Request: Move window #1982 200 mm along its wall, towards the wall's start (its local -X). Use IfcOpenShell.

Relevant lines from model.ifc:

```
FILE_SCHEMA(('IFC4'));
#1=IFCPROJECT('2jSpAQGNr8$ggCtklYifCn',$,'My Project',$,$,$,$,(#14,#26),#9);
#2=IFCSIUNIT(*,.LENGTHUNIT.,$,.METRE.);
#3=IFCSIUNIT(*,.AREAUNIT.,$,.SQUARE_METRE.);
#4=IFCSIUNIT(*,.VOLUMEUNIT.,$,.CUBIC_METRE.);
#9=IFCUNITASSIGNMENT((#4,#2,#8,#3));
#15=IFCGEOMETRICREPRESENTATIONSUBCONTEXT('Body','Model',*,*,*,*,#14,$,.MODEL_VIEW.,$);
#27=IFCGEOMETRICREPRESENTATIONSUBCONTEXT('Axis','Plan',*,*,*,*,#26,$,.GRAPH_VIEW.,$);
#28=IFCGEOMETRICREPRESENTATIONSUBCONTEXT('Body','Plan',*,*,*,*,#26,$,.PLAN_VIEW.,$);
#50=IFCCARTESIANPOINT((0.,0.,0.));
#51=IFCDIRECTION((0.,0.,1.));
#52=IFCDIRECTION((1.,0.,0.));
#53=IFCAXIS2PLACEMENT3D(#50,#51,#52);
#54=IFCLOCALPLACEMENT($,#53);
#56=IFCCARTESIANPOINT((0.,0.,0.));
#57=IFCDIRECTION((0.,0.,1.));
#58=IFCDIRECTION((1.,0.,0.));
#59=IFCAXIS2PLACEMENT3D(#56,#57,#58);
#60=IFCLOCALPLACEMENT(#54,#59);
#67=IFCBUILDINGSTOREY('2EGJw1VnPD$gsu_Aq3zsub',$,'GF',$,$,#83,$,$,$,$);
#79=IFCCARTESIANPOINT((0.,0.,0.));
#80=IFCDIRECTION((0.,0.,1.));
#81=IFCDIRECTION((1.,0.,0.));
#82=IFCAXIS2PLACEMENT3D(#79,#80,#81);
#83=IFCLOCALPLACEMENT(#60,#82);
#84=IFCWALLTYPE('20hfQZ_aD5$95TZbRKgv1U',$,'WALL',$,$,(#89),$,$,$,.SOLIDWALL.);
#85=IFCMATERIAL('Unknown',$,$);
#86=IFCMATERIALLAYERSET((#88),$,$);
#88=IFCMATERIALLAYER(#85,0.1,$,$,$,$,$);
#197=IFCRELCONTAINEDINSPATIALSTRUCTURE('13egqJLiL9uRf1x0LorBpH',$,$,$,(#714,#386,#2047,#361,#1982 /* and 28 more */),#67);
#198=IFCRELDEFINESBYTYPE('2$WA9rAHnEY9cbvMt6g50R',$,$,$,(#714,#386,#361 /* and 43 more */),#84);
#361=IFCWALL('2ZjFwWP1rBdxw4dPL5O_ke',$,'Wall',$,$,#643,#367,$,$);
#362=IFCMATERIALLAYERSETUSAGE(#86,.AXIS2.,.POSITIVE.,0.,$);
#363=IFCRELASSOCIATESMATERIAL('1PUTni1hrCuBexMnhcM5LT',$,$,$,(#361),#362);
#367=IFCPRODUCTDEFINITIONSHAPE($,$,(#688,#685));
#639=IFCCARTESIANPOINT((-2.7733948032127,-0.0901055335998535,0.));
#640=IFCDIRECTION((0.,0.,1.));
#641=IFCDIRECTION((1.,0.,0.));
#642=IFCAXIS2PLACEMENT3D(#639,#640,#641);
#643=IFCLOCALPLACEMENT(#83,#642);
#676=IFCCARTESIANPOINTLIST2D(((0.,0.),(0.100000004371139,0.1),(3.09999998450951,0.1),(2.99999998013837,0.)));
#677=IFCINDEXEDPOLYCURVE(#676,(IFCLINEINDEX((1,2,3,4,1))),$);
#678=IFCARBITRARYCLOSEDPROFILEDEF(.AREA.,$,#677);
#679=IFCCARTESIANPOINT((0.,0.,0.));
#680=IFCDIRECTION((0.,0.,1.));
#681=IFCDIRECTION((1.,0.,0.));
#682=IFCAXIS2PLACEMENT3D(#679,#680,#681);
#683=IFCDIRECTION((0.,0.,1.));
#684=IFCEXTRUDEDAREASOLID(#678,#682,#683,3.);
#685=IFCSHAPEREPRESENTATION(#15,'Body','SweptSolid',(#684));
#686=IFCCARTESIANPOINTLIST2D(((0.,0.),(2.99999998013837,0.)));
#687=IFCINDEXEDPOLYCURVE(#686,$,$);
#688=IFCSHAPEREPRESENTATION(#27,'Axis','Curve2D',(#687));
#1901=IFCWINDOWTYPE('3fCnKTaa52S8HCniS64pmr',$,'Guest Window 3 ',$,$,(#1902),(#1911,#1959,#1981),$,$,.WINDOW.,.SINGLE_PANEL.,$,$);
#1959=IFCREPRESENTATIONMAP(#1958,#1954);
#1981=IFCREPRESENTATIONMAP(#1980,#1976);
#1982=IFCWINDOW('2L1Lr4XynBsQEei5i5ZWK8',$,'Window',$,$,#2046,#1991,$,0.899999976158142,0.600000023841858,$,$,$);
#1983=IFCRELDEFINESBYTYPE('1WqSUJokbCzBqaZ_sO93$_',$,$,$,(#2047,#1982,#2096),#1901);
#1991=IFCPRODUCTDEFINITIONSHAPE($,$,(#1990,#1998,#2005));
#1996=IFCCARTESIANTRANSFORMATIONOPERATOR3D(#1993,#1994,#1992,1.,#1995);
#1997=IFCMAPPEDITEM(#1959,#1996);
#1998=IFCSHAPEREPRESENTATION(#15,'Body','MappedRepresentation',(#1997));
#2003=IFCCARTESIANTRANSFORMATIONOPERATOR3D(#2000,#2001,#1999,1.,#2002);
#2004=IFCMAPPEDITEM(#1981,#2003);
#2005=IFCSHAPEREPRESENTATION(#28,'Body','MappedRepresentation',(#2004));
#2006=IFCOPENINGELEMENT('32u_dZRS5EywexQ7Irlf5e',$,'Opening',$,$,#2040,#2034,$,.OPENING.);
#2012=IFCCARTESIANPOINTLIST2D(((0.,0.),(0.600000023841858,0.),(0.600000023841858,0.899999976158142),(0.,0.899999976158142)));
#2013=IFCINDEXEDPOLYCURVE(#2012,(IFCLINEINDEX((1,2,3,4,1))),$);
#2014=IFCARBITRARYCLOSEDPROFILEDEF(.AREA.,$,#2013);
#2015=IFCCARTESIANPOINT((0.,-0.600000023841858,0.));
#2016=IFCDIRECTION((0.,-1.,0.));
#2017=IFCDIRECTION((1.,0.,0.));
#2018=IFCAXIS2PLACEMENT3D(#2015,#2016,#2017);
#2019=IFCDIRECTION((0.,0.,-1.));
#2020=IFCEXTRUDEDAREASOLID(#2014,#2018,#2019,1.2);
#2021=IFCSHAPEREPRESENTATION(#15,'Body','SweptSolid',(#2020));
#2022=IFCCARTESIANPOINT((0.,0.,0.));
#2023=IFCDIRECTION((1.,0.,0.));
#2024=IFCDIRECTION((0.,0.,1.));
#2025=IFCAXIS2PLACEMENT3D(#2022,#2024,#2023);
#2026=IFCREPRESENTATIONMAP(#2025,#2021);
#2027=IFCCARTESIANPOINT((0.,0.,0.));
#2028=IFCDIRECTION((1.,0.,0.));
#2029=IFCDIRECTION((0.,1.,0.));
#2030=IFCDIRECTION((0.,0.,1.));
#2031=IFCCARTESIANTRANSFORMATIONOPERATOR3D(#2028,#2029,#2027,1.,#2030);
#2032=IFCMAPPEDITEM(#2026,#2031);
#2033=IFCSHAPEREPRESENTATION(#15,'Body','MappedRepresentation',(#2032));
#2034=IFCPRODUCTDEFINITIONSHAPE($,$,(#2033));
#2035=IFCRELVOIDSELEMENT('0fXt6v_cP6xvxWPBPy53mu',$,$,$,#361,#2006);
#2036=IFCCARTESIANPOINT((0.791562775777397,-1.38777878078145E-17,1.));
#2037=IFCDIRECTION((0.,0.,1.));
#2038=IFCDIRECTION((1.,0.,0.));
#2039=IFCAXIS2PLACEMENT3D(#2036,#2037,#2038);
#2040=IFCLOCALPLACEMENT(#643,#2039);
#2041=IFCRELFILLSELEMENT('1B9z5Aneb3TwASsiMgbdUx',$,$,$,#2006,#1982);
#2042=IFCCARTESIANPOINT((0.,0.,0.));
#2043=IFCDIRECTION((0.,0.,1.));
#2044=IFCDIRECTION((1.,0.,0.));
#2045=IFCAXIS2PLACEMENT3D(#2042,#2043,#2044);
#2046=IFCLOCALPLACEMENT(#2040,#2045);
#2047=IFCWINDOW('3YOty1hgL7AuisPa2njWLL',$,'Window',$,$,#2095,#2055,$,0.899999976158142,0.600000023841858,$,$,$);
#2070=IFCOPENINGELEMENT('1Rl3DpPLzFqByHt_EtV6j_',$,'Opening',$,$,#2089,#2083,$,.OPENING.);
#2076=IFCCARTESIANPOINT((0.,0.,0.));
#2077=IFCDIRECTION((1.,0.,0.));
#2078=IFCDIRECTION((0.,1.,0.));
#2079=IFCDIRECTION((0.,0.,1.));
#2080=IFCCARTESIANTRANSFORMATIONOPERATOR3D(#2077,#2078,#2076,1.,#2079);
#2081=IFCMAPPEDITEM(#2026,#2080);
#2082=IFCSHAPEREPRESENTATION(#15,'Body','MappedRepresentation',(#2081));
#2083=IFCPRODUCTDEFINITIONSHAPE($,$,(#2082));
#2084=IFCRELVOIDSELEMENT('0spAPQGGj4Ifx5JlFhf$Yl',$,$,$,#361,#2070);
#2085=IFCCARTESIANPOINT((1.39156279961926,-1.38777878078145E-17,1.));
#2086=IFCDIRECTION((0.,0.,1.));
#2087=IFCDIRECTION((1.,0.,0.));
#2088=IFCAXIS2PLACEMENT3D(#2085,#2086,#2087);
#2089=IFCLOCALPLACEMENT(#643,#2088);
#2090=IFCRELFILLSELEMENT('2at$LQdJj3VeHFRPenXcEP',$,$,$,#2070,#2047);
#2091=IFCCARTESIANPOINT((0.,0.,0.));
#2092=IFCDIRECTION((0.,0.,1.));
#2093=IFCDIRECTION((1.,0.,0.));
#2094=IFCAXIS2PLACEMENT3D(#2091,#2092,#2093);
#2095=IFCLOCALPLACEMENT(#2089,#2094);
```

```python
import ifcopenshell
import ifcopenshell.api.geometry
import ifcopenshell.util.placement

model = ifcopenshell.open("model.ifc")

window = model.by_guid("2L1Lr4XynBsQEei5i5ZWK8")
opening = window.FillsVoids[0].RelatingOpeningElement
wall = opening.VoidsElements[0].RelatingBuildingElement

wall_matrix = ifcopenshell.util.placement.get_local_placement(wall.ObjectPlacement)
shift = wall_matrix[:3, 0] * -0.2
before = ifcopenshell.util.placement.get_local_placement(window.ObjectPlacement)[:3, 3].copy()

# The window is placed relative to its opening, so it follows when the opening moves.
matrix = ifcopenshell.util.placement.get_local_placement(opening.ObjectPlacement)
matrix[:3, 3] += shift
ifcopenshell.api.geometry.edit_object_placement(
    model, product=opening, matrix=matrix, is_si=False, should_transform_children=True
)

after = ifcopenshell.util.placement.get_local_placement(window.ObjectPlacement)[:3, 3]
print("window moved by", (after - before).round(3) + 0.0)

model.write("model_v2.ifc")
```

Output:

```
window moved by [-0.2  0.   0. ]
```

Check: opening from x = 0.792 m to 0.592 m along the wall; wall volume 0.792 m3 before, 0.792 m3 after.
